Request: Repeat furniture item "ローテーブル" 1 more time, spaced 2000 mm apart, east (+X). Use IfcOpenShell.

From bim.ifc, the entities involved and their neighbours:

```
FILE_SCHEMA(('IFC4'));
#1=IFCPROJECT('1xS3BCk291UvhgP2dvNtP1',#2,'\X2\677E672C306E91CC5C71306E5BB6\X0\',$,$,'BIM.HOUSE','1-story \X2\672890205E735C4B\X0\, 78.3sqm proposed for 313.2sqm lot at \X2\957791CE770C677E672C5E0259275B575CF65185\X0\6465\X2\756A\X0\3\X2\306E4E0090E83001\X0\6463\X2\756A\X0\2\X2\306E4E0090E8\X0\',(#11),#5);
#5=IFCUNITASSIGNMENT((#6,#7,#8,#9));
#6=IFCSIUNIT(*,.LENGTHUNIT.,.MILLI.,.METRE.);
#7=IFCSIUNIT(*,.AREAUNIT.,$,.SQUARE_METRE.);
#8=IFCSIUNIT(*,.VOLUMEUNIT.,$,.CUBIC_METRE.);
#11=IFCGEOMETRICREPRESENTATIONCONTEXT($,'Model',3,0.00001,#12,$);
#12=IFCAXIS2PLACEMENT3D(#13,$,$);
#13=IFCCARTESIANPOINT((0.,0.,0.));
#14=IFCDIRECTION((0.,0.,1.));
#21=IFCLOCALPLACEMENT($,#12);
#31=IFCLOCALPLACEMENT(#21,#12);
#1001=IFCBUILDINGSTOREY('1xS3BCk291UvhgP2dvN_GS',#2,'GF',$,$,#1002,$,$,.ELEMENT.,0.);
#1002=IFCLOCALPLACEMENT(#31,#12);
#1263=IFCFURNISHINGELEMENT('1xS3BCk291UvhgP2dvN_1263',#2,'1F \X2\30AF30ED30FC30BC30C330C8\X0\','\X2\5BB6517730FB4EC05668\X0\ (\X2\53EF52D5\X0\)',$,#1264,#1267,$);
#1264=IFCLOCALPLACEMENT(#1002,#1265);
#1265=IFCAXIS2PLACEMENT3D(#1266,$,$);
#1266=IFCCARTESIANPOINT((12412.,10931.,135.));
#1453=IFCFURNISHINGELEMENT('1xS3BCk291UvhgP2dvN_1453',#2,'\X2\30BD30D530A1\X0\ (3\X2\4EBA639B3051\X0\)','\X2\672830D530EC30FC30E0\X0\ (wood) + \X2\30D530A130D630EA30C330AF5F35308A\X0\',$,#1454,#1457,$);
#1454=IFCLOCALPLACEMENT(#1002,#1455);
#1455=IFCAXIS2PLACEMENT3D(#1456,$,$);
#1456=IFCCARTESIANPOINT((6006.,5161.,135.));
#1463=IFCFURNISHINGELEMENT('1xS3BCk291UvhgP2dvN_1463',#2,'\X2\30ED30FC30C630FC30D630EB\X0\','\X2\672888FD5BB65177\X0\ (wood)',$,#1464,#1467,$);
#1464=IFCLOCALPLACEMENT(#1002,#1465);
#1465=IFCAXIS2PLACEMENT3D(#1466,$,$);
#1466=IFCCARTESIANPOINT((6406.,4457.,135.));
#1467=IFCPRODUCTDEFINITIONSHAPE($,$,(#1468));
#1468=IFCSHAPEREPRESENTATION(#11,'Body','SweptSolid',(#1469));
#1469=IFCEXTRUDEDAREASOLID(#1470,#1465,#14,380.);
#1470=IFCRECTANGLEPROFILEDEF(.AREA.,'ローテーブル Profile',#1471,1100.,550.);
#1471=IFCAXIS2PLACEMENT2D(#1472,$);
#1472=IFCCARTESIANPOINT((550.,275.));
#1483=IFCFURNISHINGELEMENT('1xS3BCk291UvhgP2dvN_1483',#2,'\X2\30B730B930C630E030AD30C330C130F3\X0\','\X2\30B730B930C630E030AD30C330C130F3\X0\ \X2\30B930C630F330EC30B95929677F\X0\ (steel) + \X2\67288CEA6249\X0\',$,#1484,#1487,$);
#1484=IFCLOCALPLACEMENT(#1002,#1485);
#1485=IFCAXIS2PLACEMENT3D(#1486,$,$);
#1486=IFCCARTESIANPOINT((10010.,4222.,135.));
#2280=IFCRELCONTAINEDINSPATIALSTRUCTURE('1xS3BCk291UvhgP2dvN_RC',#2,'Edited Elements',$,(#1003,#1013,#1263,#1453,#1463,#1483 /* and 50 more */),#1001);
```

```python
import numpy as np
import ifcopenshell
import ifcopenshell.api.geometry
import ifcopenshell.api.root
import ifcopenshell.util.element
import ifcopenshell.util.placement

model = ifcopenshell.open("bim.ifc")


def reuse_history(source, copy):
    """copy_class also copies each property set's owner history, people and application; keep the originals."""
    for rel in copy.IsDefinedBy:
        if rel.is_a("IfcRelDefinesByProperties") and (history := rel.RelatingPropertyDefinition.OwnerHistory):
            rel.RelatingPropertyDefinition.OwnerHistory = source.OwnerHistory
            ifcopenshell.util.element.remove_deep2(model, history)


source = model.by_guid("1xS3BCk291UvhgP2dvN_1463")
base = ifcopenshell.util.placement.get_local_placement(source.ObjectPlacement)
step = np.array([1.0, 0.0, 0.0]) * 2000.0

for i in range(1, 2):
    copy = ifcopenshell.api.root.copy_class(model, product=source)
    copy.Representation = ifcopenshell.util.element.copy_deep(
        model, source.Representation, exclude=["IfcGeometricRepresentationContext", "IfcRepresentationMap"]
    )
    reuse_history(source, copy)
    matrix = base.copy()
    matrix[:3, 3] += i * step
    print("added at", matrix[:3, 3].round(3) + 0.0)
    ifcopenshell.api.geometry.edit_object_placement(model, product=copy, matrix=matrix, is_si=False)

model.write("bim_v2.ifc")
```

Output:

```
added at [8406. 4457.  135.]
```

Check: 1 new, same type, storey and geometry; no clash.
